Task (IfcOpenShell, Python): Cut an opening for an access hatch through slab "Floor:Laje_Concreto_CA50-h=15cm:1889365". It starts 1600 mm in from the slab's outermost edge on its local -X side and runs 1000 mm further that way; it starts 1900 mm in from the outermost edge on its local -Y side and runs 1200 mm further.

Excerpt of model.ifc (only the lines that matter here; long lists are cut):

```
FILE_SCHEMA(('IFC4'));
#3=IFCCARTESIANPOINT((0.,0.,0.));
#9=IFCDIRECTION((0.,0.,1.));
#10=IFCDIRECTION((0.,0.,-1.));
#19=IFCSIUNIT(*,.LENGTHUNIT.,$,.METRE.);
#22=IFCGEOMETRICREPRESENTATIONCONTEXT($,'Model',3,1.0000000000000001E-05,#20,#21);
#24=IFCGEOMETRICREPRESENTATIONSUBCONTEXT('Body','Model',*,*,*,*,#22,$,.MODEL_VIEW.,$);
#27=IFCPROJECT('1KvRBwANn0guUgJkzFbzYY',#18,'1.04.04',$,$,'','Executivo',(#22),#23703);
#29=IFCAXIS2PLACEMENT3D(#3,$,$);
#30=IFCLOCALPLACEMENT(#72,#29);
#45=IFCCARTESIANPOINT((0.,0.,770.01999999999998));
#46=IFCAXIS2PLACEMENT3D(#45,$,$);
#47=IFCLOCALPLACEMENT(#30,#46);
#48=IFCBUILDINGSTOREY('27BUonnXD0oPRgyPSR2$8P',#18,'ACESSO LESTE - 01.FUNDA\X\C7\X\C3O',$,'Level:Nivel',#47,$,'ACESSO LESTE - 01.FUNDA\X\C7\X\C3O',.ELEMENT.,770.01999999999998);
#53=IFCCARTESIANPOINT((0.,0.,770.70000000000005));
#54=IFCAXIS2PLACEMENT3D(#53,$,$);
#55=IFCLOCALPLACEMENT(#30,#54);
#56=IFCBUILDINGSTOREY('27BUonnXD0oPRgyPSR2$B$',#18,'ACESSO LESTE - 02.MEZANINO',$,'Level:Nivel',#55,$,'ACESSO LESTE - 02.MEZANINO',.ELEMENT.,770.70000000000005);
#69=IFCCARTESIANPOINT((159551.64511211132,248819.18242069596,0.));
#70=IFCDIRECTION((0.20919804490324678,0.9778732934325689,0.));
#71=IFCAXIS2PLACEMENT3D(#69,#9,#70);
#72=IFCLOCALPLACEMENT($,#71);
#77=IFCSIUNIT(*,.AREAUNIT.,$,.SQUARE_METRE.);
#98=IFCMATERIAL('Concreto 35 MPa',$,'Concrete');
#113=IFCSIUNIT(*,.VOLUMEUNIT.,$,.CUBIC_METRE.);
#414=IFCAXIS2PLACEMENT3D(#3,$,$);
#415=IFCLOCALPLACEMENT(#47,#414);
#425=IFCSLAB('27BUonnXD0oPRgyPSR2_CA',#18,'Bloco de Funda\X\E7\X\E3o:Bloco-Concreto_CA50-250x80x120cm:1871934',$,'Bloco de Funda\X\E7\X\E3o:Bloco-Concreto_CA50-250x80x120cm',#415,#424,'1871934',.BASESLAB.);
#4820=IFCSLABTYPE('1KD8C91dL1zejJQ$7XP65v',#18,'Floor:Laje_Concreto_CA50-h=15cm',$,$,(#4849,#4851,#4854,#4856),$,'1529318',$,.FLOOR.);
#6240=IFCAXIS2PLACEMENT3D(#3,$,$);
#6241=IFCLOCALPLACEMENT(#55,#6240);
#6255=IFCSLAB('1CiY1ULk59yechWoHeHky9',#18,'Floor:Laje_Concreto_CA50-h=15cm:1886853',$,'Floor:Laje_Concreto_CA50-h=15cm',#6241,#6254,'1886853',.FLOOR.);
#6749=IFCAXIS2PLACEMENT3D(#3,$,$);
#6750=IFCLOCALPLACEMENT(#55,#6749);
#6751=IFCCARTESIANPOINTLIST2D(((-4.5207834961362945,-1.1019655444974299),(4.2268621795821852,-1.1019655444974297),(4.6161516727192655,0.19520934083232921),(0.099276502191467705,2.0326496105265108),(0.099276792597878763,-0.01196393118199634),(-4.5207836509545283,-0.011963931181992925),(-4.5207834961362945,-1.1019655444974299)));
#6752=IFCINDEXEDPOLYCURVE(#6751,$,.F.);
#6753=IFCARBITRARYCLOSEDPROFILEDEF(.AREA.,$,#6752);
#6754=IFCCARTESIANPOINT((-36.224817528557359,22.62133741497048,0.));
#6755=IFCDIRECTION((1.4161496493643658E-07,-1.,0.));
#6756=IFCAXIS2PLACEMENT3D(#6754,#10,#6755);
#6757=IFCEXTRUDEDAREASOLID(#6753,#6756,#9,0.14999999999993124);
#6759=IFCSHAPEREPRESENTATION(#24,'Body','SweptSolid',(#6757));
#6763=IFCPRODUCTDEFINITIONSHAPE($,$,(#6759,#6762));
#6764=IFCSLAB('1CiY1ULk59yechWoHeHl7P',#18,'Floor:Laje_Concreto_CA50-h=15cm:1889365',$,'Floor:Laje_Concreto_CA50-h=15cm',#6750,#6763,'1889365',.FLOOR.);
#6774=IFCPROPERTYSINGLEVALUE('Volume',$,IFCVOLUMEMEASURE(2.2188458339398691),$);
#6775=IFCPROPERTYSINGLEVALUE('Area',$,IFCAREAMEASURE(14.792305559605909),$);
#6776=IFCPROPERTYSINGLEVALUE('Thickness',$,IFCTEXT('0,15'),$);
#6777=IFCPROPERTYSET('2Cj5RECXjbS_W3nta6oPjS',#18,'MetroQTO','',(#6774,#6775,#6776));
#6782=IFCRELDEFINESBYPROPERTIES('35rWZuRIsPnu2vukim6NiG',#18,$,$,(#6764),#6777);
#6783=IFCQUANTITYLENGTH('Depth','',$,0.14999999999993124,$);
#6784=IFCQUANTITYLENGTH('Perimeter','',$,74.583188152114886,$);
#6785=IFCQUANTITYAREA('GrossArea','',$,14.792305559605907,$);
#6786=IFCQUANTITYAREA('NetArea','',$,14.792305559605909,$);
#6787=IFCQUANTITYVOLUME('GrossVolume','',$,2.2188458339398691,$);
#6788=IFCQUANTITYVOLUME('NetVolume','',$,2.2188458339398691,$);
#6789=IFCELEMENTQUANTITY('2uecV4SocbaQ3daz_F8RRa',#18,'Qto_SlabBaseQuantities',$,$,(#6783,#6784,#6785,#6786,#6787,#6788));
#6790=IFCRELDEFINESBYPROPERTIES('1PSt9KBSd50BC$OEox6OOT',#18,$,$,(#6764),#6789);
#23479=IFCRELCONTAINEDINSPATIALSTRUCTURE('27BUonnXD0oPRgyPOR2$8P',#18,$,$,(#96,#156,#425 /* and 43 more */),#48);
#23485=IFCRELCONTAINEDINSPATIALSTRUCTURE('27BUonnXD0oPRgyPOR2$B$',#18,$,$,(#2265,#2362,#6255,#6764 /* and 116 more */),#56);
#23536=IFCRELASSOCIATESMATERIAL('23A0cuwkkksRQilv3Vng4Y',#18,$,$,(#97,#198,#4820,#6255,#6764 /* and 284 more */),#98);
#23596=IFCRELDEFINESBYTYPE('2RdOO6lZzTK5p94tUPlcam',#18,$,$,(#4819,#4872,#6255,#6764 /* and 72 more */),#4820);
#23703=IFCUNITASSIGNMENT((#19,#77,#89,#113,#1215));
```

```python
import numpy as np
import ifcopenshell
import ifcopenshell.api.feature
import ifcopenshell.api.geometry
import ifcopenshell.api.pset
import ifcopenshell.api.root
import ifcopenshell.geom
import ifcopenshell.util.element
import ifcopenshell.util.placement
import ifcopenshell.util.representation
import ifcopenshell.util.shape
import ifcopenshell.util.unit

model = ifcopenshell.open("model.ifc")
unit_scale = ifcopenshell.util.unit.calculate_unit_scale(model)
area_scale = ifcopenshell.util.unit.calculate_unit_scale(model, "AREAUNIT")
volume_scale = ifcopenshell.util.unit.calculate_unit_scale(model, "VOLUMEUNIT")
settings = ifcopenshell.geom.settings()


def volume(element):
    """Net volume in cubic metres, openings subtracted."""
    shape = ifcopenshell.geom.create_shape(settings, element)
    return ifcopenshell.util.shape.get_volume(shape.geometry)


slab = model.by_guid("1CiY1ULk59yechWoHeHl7P")
before = volume(slab)

# Extent in the slab's own axes, in metres. The edges named are its -X and -Y sides.
slab_shape = ifcopenshell.geom.create_shape(settings, slab)
vertices = ifcopenshell.util.shape.get_vertices(slab_shape.geometry)
x_min, y_min, bottom = vertices.min(axis=0)
top = vertices[:, 2].max()

opening = ifcopenshell.api.root.create_entity(model, ifc_class="IfcOpeningElement", name="Access hatch opening", predefined_type="OPENING")
context = ifcopenshell.util.representation.get_context(model, "Model", "Body", "MODEL_VIEW")
width, depth = 1, 1.2
outline = [(0.0, 0.0), (width, 0.0), (width, depth), (0.0, depth), (0.0, 0.0)]
# Overshoot both faces by 50 mm so the cut is clean.
shape = ifcopenshell.api.geometry.add_slab_representation(
    model, context=context, depth=top - bottom + 0.1, polyline=outline
)
ifcopenshell.api.geometry.assign_representation(model, product=opening, representation=shape)

matrix = ifcopenshell.util.placement.get_local_placement(slab.ObjectPlacement)
matrix[:, 3] = matrix @ np.append(np.array([x_min + 1.6, y_min + 1.9, bottom - 0.05]) / unit_scale, 1.0)
ifcopenshell.api.geometry.edit_object_placement(model, product=opening, matrix=matrix, is_si=False)
ifcopenshell.api.feature.add_feature(model, feature=opening, element=slab)

after = volume(slab)

# Update the slab's stored quantities.
pset = model.by_id(ifcopenshell.util.element.get_pset(slab, "MetroQTO", should_inherit=False)["id"])
ifcopenshell.api.pset.edit_pset(model, pset=pset, properties={
    "Volume": model.create_entity("IfcVolumeMeasure", after / volume_scale),
    "Area": model.create_entity("IfcAreaMeasure", after / (top - bottom) / area_scale),
})
qto = model.by_id(ifcopenshell.util.element.get_pset(slab, "Qto_SlabBaseQuantities", should_inherit=False)["id"])
ifcopenshell.api.pset.edit_qto(model, qto=qto, properties={
    "NetArea": after / (top - bottom) / area_scale,
    "NetVolume": after / volume_scale,
})

print(f"slab volume {before:.3f} -> {after:.3f} m3")

model.write("model-out.ifc")
```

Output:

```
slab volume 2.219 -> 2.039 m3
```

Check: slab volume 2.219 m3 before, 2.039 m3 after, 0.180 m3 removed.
